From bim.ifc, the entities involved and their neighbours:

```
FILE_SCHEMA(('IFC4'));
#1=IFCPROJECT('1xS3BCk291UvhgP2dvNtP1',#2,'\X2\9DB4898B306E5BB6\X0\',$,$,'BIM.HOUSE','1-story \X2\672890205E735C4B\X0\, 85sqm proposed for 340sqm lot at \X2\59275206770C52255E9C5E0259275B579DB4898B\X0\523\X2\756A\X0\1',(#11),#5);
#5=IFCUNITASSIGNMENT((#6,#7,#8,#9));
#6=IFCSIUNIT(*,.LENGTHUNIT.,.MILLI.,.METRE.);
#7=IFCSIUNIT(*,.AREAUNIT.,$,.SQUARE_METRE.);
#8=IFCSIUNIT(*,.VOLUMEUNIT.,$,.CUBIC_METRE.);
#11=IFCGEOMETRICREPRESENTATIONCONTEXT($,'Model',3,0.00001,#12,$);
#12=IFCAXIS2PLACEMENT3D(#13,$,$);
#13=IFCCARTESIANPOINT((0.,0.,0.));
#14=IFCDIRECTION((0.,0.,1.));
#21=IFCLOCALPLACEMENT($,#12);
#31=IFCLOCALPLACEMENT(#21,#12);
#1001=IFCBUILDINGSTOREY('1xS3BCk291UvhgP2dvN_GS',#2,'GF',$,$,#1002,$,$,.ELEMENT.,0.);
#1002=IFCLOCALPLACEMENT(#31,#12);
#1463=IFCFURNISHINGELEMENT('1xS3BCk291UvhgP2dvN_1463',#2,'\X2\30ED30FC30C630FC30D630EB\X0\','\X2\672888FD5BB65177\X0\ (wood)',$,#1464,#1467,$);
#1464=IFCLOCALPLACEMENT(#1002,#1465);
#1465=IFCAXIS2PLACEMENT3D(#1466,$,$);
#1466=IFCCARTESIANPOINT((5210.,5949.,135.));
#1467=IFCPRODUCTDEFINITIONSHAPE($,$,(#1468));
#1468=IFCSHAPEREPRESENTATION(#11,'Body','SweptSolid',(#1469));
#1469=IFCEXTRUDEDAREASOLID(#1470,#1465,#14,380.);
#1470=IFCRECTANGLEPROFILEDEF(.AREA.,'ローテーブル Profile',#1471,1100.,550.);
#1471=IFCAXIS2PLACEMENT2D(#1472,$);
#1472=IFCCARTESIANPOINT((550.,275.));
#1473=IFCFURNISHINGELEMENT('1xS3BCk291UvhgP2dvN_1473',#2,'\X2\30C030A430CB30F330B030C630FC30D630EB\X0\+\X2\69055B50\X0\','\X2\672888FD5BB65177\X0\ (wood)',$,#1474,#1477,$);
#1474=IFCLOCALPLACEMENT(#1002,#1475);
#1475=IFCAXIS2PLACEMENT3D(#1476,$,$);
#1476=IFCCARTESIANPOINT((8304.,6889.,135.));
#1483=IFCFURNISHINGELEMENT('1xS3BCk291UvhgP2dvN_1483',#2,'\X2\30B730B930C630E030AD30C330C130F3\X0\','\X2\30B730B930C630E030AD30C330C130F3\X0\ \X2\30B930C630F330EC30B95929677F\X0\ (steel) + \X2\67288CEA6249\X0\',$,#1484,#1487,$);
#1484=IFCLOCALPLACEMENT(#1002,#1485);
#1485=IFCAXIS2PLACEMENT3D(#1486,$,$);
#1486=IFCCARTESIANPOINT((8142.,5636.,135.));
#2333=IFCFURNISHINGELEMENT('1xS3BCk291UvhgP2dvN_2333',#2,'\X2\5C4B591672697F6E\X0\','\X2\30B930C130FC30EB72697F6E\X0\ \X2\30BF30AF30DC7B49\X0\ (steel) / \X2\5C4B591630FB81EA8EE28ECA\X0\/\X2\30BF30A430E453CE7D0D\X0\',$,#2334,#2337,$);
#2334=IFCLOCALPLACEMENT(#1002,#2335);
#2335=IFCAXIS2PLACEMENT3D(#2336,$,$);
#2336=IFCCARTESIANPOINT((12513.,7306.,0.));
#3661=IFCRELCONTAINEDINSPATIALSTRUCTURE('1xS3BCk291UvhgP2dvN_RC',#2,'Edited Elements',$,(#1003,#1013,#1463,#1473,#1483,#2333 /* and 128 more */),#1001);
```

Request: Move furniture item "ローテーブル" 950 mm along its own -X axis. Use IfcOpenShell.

```python
import ifcopenshell
import ifcopenshell.api.geometry
import ifcopenshell.util.placement
import ifcopenshell.util.unit

model = ifcopenshell.open("bim.ifc")
unit_scale = ifcopenshell.util.unit.calculate_unit_scale(model)

item = model.by_id(1463)
matrix = ifcopenshell.util.placement.get_local_placement(item.ObjectPlacement)
matrix[:3, 3] -= matrix[:3, 0] * 0.95 / unit_scale
ifcopenshell.api.geometry.edit_object_placement(model, product=item, matrix=matrix, is_si=False)

print(ifcopenshell.util.placement.get_local_placement(item.ObjectPlacement).round(3) + 0.0)

model.write("bim_rev.ifc")
```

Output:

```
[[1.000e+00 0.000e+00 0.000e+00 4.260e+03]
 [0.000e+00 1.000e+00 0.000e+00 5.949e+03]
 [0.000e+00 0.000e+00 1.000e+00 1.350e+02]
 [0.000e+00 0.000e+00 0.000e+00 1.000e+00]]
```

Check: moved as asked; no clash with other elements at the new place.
